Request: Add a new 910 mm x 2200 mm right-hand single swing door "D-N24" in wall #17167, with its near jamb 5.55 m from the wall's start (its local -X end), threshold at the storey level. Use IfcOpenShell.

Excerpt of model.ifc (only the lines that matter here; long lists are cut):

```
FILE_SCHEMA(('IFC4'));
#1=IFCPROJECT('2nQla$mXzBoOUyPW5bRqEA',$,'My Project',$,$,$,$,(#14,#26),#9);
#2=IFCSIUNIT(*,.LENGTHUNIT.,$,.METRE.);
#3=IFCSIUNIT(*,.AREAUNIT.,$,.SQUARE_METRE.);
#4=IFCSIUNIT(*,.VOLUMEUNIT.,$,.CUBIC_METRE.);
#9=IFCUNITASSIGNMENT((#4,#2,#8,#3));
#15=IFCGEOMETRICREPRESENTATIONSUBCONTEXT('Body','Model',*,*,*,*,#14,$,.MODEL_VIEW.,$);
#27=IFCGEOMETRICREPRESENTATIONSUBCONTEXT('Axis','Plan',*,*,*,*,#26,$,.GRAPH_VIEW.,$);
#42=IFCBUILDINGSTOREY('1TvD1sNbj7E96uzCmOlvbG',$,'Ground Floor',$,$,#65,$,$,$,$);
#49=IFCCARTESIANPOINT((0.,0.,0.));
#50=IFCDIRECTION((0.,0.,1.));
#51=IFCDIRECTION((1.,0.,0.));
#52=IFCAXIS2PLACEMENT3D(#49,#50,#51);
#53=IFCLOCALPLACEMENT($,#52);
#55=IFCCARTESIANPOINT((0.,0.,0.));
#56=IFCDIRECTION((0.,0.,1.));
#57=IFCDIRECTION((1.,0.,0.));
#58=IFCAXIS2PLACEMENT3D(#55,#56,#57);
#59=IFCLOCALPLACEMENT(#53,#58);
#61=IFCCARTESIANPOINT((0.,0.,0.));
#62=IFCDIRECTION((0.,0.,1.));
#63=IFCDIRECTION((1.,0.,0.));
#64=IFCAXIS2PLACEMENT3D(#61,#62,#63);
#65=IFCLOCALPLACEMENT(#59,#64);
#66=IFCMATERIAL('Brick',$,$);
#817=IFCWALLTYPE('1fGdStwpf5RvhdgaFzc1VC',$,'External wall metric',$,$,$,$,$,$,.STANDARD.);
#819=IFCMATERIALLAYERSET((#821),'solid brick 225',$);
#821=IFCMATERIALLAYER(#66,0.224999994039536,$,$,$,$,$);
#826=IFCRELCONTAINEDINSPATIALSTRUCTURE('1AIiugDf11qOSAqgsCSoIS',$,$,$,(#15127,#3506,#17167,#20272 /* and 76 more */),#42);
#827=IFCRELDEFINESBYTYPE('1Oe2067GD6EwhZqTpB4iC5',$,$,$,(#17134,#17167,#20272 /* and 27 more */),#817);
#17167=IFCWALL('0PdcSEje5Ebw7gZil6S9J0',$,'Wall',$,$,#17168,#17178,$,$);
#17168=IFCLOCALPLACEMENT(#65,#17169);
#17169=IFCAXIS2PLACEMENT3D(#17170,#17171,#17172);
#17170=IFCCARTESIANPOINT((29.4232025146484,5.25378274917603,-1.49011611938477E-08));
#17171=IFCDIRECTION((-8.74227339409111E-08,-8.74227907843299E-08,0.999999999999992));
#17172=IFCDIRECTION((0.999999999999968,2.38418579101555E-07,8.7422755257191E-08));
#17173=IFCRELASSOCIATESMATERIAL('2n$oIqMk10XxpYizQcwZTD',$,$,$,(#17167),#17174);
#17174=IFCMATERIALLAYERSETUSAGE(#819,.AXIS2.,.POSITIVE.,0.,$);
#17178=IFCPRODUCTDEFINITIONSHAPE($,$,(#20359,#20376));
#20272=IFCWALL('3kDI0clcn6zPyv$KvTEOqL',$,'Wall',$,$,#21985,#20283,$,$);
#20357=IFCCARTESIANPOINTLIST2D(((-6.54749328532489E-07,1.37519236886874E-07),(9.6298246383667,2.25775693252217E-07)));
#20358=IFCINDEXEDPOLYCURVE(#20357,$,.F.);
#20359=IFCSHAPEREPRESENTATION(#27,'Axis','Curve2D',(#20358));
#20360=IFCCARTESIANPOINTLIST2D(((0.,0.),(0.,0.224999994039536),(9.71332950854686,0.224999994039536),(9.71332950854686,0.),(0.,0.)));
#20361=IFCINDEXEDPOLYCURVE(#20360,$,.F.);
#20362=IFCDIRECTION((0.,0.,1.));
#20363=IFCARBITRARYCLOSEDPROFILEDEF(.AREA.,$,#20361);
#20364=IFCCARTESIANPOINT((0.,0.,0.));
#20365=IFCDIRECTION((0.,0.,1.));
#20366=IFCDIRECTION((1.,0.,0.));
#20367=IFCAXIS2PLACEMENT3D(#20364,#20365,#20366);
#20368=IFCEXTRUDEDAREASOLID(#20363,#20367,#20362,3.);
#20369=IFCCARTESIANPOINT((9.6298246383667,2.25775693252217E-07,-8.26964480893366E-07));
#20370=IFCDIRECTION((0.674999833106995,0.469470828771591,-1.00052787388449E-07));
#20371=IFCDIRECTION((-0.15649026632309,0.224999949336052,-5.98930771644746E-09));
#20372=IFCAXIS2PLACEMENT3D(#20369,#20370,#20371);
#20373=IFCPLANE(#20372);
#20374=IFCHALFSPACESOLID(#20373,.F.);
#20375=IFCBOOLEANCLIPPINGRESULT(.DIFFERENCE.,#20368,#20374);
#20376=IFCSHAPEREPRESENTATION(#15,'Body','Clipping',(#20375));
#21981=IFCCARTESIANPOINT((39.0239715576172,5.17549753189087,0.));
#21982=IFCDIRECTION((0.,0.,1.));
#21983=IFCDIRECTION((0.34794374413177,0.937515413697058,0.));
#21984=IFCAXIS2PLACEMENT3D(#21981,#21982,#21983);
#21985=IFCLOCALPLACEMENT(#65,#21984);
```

```python
import numpy as np
import ifcopenshell
import ifcopenshell.api.feature
import ifcopenshell.api.geometry
import ifcopenshell.api.root
import ifcopenshell.api.spatial
import ifcopenshell.geom
import ifcopenshell.util.element
import ifcopenshell.util.placement
import ifcopenshell.util.representation
import ifcopenshell.util.shape
import ifcopenshell.util.unit

model = ifcopenshell.open("model.ifc")
unit_scale = ifcopenshell.util.unit.calculate_unit_scale(model)
settings = ifcopenshell.geom.settings()


def volume(element):
    """Net volume in cubic metres, openings subtracted."""
    shape = ifcopenshell.geom.create_shape(settings, element)
    return ifcopenshell.util.shape.get_volume(shape.geometry)


wall = model.by_id(17167)
storey = ifcopenshell.util.element.get_container(wall, ifc_class="IfcBuildingStorey")
context = ifcopenshell.util.representation.get_context(model, "Model", "Body", "MODEL_VIEW")
before = volume(wall)

width, height, from_end, sill = 0.91, 2.2, 5.55, 0.0  # metres

# The wall runs along its own X axis, and the end named is its -X end.
wall_shape = ifcopenshell.geom.create_shape(settings, wall)
x, y, z = ifcopenshell.util.shape.get_vertices(wall_shape.geometry).T
start = x.min() + from_end
face, thickness = float(y.min()), float(y.max() - y.min())
wall_matrix = ifcopenshell.util.placement.get_local_placement(wall.ObjectPlacement)
level = ifcopenshell.util.placement.get_local_placement(storey.ObjectPlacement)[2, 3]


def in_wall(x, y):
    """Placement at x, y metres in the wall's axes, at sill height."""
    matrix = wall_matrix.copy()
    matrix[:, 3] = wall_matrix @ np.array([x / unit_scale, y / unit_scale, 0.0, 1.0])
    matrix[2, 3] = level + sill / unit_scale
    return matrix


# Opening: a box that overshoots both wall faces by 50 mm.
opening = ifcopenshell.api.root.create_entity(model, ifc_class="IfcOpeningElement", predefined_type="OPENING")
box = ifcopenshell.api.geometry.add_wall_representation(
    model, context=context, length=width, height=height, thickness=thickness + 0.1
)
ifcopenshell.api.geometry.assign_representation(model, product=opening, representation=box)
ifcopenshell.api.geometry.edit_object_placement(model, product=opening, matrix=in_wall(start, face - 0.05), is_si=False)
ifcopenshell.api.feature.add_feature(model, feature=opening, element=wall)

door = ifcopenshell.api.root.create_entity(model, ifc_class="IfcDoor", name="D-N24", predefined_type="DOOR")
door.OverallWidth, door.OverallHeight = width / unit_scale, height / unit_scale
door.OperationType = "SINGLE_SWING_RIGHT"
body = ifcopenshell.api.geometry.add_door_representation(
    model,
    context=context,
    overall_width=door.OverallWidth,
    overall_height=door.OverallHeight,
    operation_type="SINGLE_SWING_RIGHT",
    lining_properties={"LiningDepth": thickness / unit_scale, "ThresholdDepth": thickness / unit_scale},
)
ifcopenshell.api.geometry.assign_representation(model, product=door, representation=body)
ifcopenshell.api.spatial.assign_container(model, products=[door], relating_structure=storey)
ifcopenshell.api.feature.add_filling(model, opening=opening, element=door)

# The lining spans the wall, so the door starts at the wall face.
ifcopenshell.api.geometry.edit_object_placement(model, product=door, matrix=in_wall(start, face), is_si=False)

after = volume(wall)

print(f"wall volume {before:.3f} -> {after:.3f} m3")

model.write("model_v2.ifc")
```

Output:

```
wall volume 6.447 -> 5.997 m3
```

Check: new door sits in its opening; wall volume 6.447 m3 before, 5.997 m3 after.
